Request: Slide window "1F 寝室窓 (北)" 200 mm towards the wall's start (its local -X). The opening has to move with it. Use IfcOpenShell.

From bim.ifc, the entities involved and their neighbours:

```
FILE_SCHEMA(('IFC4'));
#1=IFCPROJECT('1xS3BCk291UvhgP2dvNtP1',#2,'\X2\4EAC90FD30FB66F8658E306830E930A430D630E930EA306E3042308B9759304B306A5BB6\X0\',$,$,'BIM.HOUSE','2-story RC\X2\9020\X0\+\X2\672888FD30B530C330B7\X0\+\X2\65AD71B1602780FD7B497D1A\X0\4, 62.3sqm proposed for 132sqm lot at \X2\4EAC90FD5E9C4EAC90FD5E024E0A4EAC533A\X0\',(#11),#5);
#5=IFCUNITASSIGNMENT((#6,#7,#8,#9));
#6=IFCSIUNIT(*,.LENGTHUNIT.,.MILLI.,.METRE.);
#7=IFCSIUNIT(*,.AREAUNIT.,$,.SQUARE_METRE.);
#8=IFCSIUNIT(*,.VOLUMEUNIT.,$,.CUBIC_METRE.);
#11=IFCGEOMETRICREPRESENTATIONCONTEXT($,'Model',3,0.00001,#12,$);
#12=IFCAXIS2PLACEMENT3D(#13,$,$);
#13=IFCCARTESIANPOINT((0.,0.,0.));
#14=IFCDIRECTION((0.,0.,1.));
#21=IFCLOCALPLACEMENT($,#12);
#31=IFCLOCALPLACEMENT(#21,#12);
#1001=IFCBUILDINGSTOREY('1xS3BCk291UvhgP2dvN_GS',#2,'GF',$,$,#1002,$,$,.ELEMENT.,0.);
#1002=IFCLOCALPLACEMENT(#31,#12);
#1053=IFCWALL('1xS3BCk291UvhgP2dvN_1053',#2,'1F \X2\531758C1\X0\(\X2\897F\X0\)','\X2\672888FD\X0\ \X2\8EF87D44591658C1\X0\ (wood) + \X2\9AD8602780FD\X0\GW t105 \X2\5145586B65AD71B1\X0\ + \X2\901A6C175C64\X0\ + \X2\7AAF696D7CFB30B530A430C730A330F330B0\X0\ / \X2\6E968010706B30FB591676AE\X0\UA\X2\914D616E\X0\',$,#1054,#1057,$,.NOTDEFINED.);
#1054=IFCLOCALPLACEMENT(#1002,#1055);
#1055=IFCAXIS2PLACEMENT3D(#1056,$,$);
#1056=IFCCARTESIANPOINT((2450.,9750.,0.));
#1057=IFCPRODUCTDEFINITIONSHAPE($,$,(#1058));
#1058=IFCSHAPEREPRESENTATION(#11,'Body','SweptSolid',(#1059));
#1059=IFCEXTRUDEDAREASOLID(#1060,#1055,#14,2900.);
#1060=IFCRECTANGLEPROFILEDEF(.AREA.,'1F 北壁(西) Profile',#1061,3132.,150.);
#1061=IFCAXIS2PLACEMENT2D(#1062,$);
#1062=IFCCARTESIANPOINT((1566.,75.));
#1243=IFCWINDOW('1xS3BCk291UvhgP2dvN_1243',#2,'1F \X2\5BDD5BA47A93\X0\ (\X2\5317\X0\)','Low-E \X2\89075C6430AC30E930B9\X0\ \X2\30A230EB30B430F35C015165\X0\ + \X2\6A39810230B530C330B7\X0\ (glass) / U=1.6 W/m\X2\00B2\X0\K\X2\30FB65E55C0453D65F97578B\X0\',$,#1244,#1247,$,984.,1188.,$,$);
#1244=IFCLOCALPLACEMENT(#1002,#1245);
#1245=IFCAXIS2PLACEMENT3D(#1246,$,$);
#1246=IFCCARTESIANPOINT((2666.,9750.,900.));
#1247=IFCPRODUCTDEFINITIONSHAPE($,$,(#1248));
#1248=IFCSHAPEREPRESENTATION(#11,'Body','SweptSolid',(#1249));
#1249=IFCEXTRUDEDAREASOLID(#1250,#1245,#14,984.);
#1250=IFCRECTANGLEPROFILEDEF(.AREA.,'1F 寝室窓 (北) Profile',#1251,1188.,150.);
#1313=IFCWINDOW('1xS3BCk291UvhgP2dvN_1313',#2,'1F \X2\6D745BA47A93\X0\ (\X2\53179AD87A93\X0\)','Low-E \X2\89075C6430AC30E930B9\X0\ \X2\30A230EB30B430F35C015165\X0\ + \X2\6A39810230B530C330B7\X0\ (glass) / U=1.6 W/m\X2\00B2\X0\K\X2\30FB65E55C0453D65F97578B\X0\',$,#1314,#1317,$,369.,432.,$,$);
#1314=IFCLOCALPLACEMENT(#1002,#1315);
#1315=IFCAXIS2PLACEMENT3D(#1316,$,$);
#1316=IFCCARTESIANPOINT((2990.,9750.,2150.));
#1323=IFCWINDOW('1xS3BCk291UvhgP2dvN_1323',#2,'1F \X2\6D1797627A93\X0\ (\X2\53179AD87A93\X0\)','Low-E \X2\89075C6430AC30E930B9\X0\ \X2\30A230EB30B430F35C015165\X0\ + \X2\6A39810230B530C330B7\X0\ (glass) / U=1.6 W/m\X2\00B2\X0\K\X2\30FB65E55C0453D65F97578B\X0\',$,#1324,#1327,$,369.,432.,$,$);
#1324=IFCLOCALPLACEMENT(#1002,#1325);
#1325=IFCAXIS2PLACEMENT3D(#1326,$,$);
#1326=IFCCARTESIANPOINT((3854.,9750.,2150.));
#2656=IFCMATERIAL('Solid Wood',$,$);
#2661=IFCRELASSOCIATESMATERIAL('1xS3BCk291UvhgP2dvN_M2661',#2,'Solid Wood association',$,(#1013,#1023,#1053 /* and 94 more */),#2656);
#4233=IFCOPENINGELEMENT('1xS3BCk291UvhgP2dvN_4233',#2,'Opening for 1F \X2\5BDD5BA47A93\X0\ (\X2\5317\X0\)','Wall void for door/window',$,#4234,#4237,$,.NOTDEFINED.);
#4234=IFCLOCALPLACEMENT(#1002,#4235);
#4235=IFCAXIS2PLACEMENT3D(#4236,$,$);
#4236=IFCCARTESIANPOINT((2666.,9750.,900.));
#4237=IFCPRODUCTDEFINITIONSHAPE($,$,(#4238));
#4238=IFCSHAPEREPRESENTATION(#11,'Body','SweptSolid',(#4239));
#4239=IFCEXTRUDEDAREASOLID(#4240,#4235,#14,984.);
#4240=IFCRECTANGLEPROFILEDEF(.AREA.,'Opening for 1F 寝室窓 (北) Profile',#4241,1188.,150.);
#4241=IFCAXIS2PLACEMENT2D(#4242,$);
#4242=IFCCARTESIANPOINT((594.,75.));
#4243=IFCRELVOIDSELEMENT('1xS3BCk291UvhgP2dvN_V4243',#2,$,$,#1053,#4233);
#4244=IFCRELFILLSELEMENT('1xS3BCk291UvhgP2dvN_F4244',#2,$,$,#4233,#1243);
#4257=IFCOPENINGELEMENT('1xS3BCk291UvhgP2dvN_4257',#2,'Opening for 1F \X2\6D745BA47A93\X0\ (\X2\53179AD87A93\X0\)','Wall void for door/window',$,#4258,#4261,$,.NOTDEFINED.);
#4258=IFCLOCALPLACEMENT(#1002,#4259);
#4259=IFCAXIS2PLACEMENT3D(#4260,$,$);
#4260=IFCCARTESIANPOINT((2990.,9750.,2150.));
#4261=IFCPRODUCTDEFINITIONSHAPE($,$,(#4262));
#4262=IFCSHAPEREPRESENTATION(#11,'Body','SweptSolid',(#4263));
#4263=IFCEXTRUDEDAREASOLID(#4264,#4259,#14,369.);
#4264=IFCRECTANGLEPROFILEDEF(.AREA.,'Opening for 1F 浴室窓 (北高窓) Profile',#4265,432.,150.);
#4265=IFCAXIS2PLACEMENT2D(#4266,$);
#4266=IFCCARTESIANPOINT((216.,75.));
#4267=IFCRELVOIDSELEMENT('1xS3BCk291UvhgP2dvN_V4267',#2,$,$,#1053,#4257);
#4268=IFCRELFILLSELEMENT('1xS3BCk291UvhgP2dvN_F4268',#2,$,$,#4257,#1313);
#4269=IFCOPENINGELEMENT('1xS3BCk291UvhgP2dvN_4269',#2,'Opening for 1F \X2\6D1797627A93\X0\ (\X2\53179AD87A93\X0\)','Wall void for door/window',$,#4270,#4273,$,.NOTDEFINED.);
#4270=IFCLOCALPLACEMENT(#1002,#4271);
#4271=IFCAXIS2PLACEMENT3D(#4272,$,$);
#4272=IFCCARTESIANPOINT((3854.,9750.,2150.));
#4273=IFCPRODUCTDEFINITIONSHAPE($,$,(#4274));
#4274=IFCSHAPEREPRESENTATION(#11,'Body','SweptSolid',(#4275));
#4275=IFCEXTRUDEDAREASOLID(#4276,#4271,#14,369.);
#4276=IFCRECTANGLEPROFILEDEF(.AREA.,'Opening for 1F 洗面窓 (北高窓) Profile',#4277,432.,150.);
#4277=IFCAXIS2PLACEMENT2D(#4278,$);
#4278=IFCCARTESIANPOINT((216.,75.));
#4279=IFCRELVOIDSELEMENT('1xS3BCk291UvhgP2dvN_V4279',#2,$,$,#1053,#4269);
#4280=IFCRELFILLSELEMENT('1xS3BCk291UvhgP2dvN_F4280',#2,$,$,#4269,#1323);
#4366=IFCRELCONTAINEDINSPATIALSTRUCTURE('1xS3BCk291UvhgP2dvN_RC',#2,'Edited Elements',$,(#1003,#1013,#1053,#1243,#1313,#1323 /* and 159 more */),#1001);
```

```python
import ifcopenshell
import ifcopenshell.api.geometry
import ifcopenshell.util.placement

model = ifcopenshell.open("bim.ifc")

window = model.by_guid("1xS3BCk291UvhgP2dvN_1243")
opening = window.FillsVoids[0].RelatingOpeningElement
wall = opening.VoidsElements[0].RelatingBuildingElement

wall_matrix = ifcopenshell.util.placement.get_local_placement(wall.ObjectPlacement)
shift = wall_matrix[:3, 0] * -200.0
before = ifcopenshell.util.placement.get_local_placement(window.ObjectPlacement)[:3, 3].copy()

# The window is not placed relative to its opening, so move both.
for product in (opening, window):
    matrix = ifcopenshell.util.placement.get_local_placement(product.ObjectPlacement)
    matrix[:3, 3] += shift
    ifcopenshell.api.geometry.edit_object_placement(model, product=product, matrix=matrix, is_si=False)

after = ifcopenshell.util.placement.get_local_placement(window.ObjectPlacement)[:3, 3]
print("window moved by", (after - before).round(3) + 0.0)

model.write("bim_rev.ifc")
```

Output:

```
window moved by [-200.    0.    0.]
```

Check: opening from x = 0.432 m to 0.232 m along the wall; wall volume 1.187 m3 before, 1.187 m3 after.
